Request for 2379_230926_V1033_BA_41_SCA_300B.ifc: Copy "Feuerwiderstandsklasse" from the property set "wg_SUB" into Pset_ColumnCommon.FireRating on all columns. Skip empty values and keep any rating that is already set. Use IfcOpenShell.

First a look at what the model holds.

```python
import ifcopenshell
import ifcopenshell.util.element

model = ifcopenshell.open("2379_230926_V1033_BA_41_SCA_300B.ifc")
print(model.schema)
columns = model.by_type("IfcColumn")
print(len(columns), "columns")
for e in columns[:8]:
    source = ifcopenshell.util.element.get_pset(e, "wg_SUB", "Feuerwiderstandsklasse")
    target = ifcopenshell.util.element.get_pset(e, "Pset_ColumnCommon", "FireRating")
    print(e.id(), repr(source), repr(target), sep=" | ")
```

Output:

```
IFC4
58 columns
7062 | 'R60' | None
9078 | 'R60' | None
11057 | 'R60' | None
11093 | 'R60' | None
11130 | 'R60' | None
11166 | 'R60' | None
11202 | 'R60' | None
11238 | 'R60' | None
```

```python
import ifcopenshell
import ifcopenshell.api.pset
import ifcopenshell.util.element

model = ifcopenshell.open("2379_230926_V1033_BA_41_SCA_300B.ifc")

count = 0
for e in model.by_type("IfcColumn"):
    value = ifcopenshell.util.element.get_pset(e, "wg_SUB", "Feuerwiderstandsklasse")
    current = ifcopenshell.util.element.get_pset(e, "Pset_ColumnCommon", "FireRating")
    if not value or not value.strip() or current:
        continue
    # add_pset returns the element's existing set when there is one.
    pset = ifcopenshell.api.pset.add_pset(model, product=e, name="Pset_ColumnCommon")
    ifcopenshell.api.pset.edit_pset(model, pset=pset, properties={"FireRating": value})
    count += 1

print(count, "columns updated")

model.write("2379_230926_V1033_BA_41_SCA_300B_rev.ifc")
```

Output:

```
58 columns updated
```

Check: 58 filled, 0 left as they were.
